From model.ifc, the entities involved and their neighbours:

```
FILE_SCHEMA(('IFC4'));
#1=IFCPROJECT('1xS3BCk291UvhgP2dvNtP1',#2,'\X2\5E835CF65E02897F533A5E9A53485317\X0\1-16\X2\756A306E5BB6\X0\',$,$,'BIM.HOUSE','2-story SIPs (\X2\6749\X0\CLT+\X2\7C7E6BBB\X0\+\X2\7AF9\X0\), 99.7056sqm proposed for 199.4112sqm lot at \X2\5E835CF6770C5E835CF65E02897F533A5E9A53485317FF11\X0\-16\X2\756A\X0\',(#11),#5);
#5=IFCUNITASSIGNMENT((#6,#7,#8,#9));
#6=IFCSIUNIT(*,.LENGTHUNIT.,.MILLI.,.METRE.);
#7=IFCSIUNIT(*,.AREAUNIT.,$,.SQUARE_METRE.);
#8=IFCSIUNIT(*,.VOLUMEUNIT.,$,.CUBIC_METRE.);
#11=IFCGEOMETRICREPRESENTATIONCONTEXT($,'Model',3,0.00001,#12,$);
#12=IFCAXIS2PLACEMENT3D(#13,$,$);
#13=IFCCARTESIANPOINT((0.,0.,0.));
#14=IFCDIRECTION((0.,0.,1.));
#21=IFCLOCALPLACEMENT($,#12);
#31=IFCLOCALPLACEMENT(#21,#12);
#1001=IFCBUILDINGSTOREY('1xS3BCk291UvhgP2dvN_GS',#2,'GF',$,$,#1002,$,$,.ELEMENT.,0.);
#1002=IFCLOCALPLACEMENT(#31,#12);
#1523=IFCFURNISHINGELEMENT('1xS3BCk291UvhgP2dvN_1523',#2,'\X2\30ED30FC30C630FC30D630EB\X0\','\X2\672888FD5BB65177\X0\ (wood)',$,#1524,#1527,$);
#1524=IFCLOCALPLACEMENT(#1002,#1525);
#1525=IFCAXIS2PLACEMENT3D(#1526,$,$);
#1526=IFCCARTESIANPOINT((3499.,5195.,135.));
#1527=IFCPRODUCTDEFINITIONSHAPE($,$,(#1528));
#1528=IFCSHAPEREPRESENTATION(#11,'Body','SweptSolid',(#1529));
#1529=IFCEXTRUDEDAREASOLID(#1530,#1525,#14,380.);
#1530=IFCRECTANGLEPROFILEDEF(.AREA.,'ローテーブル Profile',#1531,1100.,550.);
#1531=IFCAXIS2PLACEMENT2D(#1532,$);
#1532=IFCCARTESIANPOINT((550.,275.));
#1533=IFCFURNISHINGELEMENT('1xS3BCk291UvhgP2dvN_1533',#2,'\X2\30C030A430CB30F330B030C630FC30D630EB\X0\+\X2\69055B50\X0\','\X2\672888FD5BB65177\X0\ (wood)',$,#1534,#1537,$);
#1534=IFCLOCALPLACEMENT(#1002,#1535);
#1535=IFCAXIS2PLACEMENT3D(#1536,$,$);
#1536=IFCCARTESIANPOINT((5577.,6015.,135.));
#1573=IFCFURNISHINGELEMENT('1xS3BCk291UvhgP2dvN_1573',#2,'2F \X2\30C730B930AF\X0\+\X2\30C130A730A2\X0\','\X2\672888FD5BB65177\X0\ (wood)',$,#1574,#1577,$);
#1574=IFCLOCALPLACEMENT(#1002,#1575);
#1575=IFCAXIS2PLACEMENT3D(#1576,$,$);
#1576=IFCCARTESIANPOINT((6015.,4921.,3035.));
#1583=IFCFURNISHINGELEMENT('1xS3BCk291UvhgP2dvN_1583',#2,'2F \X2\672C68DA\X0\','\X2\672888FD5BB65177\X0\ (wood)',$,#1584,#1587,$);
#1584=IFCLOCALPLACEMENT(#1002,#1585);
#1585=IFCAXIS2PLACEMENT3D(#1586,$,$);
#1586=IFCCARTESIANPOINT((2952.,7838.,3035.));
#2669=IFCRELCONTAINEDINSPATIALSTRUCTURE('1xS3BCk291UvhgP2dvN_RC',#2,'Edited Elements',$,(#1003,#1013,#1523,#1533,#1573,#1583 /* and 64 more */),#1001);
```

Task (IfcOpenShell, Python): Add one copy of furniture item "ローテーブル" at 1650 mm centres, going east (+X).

```python
import numpy as np
import ifcopenshell
import ifcopenshell.api.geometry
import ifcopenshell.api.root
import ifcopenshell.util.element
import ifcopenshell.util.placement
import ifcopenshell.util.unit

model = ifcopenshell.open("model.ifc")
unit_scale = ifcopenshell.util.unit.calculate_unit_scale(model)


def reuse_history(source, copy):
    """copy_class also copies each property set's owner history, people and application; keep the originals."""
    for rel in copy.IsDefinedBy:
        if rel.is_a("IfcRelDefinesByProperties") and (history := rel.RelatingPropertyDefinition.OwnerHistory):
            rel.RelatingPropertyDefinition.OwnerHistory = source.OwnerHistory
            ifcopenshell.util.element.remove_deep2(model, history)


source = model.by_id(1523)
base = ifcopenshell.util.placement.get_local_placement(source.ObjectPlacement)
step = np.array([1.0, 0.0, 0.0]) * 1.65 / unit_scale

for i in range(1, 2):
    copy = ifcopenshell.api.root.copy_class(model, product=source)
    copy.Representation = ifcopenshell.util.element.copy_deep(
        model, source.Representation, exclude=["IfcGeometricRepresentationContext", "IfcRepresentationMap"]
    )
    reuse_history(source, copy)
    matrix = base.copy()
    matrix[:3, 3] += i * step
    print("added at", matrix[:3, 3].round(3) + 0.0)
    ifcopenshell.api.geometry.edit_object_placement(model, product=copy, matrix=matrix, is_si=False)

model.write("model_edited.ifc")
```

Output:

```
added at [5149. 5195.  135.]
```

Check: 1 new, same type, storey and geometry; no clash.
